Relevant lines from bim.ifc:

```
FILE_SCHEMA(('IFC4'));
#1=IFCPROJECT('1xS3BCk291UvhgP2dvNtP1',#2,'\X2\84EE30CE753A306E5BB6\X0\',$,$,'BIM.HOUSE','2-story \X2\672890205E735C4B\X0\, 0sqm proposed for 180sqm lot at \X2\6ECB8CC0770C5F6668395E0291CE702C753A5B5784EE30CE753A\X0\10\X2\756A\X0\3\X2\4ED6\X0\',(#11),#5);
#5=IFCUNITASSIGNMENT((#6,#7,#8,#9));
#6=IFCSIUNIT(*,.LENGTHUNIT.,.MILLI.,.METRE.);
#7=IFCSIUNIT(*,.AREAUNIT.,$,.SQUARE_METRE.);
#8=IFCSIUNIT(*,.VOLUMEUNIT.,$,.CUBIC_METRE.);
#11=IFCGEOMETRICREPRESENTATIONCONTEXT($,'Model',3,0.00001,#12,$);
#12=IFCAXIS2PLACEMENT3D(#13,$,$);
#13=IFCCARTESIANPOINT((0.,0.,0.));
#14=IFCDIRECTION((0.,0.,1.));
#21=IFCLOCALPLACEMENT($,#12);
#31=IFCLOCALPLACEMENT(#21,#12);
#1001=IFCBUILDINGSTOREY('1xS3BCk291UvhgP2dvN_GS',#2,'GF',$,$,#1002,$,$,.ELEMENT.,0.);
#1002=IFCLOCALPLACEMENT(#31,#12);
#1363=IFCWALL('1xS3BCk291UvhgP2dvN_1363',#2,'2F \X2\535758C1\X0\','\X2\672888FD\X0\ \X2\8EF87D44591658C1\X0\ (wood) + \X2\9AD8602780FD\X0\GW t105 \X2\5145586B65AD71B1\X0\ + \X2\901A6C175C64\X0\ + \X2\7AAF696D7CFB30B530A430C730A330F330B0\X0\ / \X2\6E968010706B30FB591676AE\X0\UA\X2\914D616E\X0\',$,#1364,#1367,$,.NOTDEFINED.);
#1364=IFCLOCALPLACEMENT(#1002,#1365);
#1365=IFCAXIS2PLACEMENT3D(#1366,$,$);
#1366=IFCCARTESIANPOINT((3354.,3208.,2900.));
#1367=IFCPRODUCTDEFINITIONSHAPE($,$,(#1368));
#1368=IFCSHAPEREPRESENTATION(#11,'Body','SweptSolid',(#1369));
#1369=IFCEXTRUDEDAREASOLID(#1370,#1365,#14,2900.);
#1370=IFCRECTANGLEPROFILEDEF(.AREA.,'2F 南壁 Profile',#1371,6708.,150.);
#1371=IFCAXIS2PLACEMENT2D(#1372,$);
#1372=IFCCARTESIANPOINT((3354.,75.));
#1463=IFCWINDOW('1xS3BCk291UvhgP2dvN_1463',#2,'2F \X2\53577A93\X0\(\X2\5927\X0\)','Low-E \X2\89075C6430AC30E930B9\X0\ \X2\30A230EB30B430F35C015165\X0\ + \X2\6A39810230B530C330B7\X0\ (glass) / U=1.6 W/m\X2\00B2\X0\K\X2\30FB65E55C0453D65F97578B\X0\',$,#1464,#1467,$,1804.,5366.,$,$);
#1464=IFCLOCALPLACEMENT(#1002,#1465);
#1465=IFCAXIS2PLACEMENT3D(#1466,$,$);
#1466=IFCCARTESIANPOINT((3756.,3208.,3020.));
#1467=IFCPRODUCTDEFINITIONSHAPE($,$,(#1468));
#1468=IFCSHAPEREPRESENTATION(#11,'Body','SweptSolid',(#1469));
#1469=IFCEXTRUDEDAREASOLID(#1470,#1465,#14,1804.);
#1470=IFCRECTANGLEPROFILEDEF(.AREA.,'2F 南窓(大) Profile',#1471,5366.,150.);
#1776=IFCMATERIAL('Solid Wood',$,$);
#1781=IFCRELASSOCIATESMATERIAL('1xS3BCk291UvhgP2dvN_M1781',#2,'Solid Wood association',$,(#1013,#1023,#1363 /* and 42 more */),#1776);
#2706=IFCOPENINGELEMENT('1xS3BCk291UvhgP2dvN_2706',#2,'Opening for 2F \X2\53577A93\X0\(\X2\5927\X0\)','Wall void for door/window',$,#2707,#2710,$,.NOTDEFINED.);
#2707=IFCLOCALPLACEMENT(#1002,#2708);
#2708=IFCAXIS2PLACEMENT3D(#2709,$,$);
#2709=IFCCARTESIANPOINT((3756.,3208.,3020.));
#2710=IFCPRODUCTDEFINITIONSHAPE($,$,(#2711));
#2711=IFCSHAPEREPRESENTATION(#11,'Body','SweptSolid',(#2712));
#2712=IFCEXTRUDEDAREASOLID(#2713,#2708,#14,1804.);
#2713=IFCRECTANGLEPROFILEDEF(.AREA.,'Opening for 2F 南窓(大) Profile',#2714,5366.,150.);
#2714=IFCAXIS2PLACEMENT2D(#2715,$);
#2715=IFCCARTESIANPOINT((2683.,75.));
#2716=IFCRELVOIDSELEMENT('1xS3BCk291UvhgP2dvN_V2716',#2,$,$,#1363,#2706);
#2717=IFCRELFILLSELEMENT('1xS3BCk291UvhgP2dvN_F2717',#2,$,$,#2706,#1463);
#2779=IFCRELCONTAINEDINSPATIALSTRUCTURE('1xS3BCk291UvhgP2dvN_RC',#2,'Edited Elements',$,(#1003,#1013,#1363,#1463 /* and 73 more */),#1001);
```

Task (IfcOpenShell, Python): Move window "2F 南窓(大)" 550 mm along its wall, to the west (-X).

```python
import ifcopenshell
import ifcopenshell.api.geometry
import ifcopenshell.util.placement

model = ifcopenshell.open("bim.ifc")

window = model.by_id(1463)
opening = window.FillsVoids[0].RelatingOpeningElement
wall = opening.VoidsElements[0].RelatingBuildingElement

wall_matrix = ifcopenshell.util.placement.get_local_placement(wall.ObjectPlacement)
shift = wall_matrix[:3, 0] * -550.0
before = ifcopenshell.util.placement.get_local_placement(window.ObjectPlacement)[:3, 3].copy()

# The window is not placed relative to its opening, so move both.
for product in (opening, window):
    matrix = ifcopenshell.util.placement.get_local_placement(product.ObjectPlacement)
    matrix[:3, 3] += shift
    ifcopenshell.api.geometry.edit_object_placement(model, product=product, matrix=matrix, is_si=False)

after = ifcopenshell.util.placement.get_local_placement(window.ObjectPlacement)[:3, 3]
print("window moved by", (after - before).round(3) + 0.0)

model.write("bim_rev.ifc")
```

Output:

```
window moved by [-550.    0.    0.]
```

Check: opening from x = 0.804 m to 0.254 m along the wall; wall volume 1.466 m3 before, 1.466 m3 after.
